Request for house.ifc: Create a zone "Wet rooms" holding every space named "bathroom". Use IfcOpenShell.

First a look at what the model holds.

```python
import ifcopenshell

model = ifcopenshell.open("house.ifc")
print(model.schema)
seen = {}
for space in model.by_type("IfcSpace"):
    seen[space.LongName] = seen.get(space.LongName, 0) + 1
for name, count in sorted(seen.items(), key=str):
    print(count, "x", name)
print("zones:", [z.Name for z in model.by_type("IfcZone")][:20])
```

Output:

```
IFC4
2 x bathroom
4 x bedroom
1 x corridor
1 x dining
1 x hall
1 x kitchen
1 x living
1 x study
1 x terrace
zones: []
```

```python
import ifcopenshell
import ifcopenshell.api.group
import ifcopenshell.api.root

model = ifcopenshell.open("house.ifc")

names = {"bathroom"}
spaces = [s for s in model.by_type("IfcSpace") if s.LongName in names]

zone = ifcopenshell.api.root.create_entity(model, ifc_class="IfcZone", name="Wet rooms")
ifcopenshell.api.group.assign_group(model, products=spaces, group=zone)
print(len(spaces), "spaces in", zone.Name)

model.write("house_rev.ifc")
```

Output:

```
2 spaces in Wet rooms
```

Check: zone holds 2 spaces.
